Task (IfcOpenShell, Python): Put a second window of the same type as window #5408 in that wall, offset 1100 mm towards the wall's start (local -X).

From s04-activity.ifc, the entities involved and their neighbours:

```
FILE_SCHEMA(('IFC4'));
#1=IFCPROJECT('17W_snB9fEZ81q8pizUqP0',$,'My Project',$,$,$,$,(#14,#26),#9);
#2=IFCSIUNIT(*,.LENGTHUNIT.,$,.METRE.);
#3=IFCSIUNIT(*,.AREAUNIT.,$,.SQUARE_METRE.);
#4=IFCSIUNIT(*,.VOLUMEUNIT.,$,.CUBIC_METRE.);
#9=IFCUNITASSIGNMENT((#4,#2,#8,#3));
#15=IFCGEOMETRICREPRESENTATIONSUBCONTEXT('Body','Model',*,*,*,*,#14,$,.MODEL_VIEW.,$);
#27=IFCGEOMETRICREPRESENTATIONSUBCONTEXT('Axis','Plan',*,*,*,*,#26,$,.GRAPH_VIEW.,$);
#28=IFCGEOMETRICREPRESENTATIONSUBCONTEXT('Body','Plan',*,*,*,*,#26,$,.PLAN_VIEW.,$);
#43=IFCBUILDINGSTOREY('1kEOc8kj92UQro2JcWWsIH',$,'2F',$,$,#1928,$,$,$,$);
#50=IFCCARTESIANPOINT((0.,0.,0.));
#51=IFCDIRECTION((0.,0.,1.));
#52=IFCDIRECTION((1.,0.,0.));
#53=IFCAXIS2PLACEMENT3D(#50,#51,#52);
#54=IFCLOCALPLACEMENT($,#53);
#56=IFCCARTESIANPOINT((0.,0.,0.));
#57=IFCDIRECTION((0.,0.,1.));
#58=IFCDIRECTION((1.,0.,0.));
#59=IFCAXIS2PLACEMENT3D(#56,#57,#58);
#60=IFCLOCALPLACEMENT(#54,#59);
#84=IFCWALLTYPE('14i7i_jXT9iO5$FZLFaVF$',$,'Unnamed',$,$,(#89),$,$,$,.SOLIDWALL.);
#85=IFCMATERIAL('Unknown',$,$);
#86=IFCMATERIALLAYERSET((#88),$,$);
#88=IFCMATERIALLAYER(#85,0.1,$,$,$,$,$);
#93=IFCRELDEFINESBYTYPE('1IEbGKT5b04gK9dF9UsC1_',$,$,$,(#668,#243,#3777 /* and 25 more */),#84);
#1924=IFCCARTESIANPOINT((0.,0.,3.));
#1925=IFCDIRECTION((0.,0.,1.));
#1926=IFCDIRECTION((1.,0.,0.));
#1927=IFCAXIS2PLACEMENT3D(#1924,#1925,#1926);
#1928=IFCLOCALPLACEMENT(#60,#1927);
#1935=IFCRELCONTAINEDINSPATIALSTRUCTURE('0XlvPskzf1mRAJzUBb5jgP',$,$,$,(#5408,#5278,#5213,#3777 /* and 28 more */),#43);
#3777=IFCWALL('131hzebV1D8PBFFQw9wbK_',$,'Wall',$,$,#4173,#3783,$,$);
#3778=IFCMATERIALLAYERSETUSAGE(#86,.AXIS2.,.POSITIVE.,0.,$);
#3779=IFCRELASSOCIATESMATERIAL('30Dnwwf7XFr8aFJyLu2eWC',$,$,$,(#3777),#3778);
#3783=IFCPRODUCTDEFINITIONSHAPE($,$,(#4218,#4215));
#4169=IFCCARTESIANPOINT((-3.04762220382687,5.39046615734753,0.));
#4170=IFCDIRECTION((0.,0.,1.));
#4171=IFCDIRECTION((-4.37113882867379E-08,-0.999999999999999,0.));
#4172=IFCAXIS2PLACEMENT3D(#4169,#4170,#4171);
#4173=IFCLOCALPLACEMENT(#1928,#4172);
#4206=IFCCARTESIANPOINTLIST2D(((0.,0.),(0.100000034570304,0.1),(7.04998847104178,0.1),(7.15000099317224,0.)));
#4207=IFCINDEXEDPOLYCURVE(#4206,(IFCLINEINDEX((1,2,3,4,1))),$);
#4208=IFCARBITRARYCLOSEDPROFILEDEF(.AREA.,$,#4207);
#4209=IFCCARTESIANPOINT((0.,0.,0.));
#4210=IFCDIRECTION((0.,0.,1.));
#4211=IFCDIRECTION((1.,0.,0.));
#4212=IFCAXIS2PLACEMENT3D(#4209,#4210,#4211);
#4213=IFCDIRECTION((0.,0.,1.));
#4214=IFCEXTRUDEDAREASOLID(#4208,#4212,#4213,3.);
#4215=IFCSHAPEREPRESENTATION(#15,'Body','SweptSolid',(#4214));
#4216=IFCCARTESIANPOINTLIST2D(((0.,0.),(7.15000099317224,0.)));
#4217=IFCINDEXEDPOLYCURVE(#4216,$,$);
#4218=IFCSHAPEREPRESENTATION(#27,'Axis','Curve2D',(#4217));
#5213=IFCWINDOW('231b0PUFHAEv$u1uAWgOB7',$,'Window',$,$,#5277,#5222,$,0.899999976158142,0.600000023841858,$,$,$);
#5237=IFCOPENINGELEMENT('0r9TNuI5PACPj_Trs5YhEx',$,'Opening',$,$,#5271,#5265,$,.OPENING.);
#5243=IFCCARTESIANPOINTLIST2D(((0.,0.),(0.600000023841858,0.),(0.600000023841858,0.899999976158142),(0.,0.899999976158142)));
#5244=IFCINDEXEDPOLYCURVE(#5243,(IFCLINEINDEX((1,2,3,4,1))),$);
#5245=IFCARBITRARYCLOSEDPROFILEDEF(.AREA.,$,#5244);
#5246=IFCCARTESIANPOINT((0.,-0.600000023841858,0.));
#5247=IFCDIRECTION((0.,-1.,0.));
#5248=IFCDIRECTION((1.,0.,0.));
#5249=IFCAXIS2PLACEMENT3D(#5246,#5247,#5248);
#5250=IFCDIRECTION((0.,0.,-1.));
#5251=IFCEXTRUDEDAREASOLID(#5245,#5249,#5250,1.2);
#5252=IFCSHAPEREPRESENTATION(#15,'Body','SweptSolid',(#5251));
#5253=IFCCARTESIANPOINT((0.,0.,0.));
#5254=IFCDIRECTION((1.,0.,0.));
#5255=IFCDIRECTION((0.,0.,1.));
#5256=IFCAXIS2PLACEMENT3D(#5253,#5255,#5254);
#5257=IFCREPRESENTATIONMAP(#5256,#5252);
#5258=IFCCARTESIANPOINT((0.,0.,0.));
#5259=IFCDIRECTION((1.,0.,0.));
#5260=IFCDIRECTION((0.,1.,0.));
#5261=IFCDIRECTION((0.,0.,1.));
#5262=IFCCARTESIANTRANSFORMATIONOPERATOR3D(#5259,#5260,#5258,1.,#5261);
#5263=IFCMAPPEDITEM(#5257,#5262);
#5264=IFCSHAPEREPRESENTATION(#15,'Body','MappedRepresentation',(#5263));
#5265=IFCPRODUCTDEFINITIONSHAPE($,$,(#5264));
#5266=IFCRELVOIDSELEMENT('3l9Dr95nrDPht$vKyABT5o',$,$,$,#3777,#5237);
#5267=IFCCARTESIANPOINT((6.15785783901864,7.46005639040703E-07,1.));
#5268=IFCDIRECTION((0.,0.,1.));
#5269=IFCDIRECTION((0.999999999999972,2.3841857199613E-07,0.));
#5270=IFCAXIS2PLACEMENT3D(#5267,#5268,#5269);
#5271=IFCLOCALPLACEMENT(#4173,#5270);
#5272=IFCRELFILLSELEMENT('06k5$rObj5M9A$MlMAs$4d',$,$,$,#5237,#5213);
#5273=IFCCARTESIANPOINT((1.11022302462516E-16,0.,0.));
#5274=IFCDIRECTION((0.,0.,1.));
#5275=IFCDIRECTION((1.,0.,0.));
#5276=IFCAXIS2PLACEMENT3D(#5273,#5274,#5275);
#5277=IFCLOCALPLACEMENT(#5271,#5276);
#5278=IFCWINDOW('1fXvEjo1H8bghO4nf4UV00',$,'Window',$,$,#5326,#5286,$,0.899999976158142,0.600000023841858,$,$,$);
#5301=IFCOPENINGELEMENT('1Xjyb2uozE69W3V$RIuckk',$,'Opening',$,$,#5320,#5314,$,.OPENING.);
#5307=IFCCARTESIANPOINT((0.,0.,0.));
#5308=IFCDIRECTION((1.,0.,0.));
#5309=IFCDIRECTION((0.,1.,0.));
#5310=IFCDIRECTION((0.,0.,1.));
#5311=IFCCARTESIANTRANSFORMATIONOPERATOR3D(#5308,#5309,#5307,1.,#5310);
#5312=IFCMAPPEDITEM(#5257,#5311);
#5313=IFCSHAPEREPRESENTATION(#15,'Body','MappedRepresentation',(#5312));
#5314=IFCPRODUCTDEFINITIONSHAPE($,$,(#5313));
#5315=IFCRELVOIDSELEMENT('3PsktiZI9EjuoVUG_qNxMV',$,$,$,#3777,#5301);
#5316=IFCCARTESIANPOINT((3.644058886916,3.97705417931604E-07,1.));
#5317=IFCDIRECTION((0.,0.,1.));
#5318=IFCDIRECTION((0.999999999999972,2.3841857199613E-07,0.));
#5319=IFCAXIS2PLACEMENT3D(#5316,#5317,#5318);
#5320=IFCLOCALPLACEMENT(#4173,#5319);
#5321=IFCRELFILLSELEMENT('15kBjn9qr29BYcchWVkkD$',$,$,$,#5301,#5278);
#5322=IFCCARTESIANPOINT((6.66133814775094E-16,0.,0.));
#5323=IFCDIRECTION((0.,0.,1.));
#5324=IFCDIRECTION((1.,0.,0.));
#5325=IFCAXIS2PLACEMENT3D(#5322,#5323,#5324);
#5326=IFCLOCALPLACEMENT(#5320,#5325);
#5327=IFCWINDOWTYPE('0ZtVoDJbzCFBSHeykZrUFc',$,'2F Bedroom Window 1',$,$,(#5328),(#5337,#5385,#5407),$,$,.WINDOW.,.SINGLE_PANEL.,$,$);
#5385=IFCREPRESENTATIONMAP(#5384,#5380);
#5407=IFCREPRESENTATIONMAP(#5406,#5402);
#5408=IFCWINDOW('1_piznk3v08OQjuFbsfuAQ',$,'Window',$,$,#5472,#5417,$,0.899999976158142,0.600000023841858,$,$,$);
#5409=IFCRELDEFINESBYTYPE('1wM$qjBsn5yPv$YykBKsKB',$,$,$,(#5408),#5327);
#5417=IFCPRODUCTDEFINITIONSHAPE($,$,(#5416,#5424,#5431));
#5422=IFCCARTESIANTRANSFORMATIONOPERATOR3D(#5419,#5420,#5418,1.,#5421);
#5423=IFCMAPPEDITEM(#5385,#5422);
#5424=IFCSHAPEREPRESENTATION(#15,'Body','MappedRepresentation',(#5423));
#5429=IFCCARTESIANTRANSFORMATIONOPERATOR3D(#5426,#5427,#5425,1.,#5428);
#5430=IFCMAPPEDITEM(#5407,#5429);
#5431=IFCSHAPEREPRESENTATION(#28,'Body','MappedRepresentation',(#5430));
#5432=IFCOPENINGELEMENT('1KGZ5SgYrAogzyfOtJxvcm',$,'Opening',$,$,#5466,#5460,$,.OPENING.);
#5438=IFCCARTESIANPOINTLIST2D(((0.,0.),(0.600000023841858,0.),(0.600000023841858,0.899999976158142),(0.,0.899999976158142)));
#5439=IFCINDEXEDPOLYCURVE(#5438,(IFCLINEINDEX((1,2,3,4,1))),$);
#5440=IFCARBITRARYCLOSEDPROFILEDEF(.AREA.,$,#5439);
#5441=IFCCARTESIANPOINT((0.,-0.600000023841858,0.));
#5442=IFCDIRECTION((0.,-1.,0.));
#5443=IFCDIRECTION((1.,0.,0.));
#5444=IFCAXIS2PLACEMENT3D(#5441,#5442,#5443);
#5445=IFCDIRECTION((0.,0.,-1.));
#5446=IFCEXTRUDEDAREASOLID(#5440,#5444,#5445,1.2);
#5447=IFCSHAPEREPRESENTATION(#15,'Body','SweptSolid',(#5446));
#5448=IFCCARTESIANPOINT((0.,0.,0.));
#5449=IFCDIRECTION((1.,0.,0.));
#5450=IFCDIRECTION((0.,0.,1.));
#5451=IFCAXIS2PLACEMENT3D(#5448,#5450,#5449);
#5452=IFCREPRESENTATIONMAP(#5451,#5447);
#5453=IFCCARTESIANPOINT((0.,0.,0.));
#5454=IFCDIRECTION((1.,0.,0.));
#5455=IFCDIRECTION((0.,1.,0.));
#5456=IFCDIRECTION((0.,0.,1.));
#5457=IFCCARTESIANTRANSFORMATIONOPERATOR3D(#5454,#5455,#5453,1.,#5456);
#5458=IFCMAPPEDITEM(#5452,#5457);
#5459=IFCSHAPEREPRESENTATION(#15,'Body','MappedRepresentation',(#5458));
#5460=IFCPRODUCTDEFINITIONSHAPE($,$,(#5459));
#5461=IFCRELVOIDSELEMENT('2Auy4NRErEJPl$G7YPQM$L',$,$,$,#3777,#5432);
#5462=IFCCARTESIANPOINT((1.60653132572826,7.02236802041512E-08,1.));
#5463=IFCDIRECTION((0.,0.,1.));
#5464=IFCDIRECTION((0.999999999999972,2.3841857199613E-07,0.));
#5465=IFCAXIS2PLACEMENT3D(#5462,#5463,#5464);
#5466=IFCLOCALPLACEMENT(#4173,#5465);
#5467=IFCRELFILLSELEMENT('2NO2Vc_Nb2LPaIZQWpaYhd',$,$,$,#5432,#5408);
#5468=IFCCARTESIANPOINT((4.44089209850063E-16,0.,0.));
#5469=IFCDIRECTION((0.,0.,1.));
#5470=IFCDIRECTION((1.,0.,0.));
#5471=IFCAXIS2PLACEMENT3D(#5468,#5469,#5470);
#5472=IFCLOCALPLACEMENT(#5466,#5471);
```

```python
import ifcopenshell
import ifcopenshell.api.feature
import ifcopenshell.api.geometry
import ifcopenshell.api.root
import ifcopenshell.geom
import ifcopenshell.util.element
import ifcopenshell.util.placement
import ifcopenshell.util.shape
import ifcopenshell.util.unit

model = ifcopenshell.open("s04-activity.ifc")
unit_scale = ifcopenshell.util.unit.calculate_unit_scale(model)
settings = ifcopenshell.geom.settings()


def volume(element):
    """Net volume in cubic metres, openings subtracted."""
    shape = ifcopenshell.geom.create_shape(settings, element)
    return ifcopenshell.util.shape.get_volume(shape.geometry)


window = model.by_guid("1_piznk3v08OQjuFbsfuAQ")
opening = window.FillsVoids[0].RelatingOpeningElement
wall = opening.VoidsElements[0].RelatingBuildingElement
before = volume(wall)
shift = ifcopenshell.util.placement.get_local_placement(wall.ObjectPlacement)[:3, 0] * -1.1 / unit_scale

# copy_class copies the void relationship, type, container and properties, but no geometry.
new_opening = ifcopenshell.api.root.copy_class(model, product=opening)
new_opening.Representation = ifcopenshell.util.element.copy_deep(
    model, opening.Representation, exclude=["IfcGeometricRepresentationContext", "IfcRepresentationMap"]
)
new_window = ifcopenshell.api.root.copy_class(model, product=window)
new_window.Representation = ifcopenshell.util.element.copy_deep(
    model, window.Representation, exclude=["IfcGeometricRepresentationContext", "IfcRepresentationMap"]
)
ifcopenshell.api.feature.add_filling(model, opening=new_opening, element=new_window)

for old, new in ((opening, new_opening), (window, new_window)):
    matrix = ifcopenshell.util.placement.get_local_placement(old.ObjectPlacement)
    matrix[:3, 3] += shift
    ifcopenshell.api.geometry.edit_object_placement(model, product=new, matrix=matrix, is_si=False)

after = volume(wall)

print(f"wall volume {before:.3f} -> {after:.3f} m3")

model.write("s04-activity_rev.ifc")
```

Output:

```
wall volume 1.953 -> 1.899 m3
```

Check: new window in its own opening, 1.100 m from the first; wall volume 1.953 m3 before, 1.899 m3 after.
